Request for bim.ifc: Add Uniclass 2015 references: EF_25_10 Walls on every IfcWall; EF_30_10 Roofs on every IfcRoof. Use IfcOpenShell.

First a look at what the model holds.

```python
import ifcopenshell

model = ifcopenshell.open("bim.ifc")
print(model.schema)
print("classifications:", [c.Name for c in model.by_type("IfcClassification")])
for ifc_class in ("IfcDoor", "IfcRoof", "IfcStair", "IfcWall", "IfcWindow"):
    print(ifc_class, len(model.by_type(ifc_class)))
```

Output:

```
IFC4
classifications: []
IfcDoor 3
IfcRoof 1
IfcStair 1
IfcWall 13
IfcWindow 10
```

```python
import ifcopenshell
import ifcopenshell.api.classification

model = ifcopenshell.open("bim.ifc")

system = ifcopenshell.api.classification.add_classification(model, classification="Uniclass 2015")

codes = {
    "IfcWall": ("EF_25_10", "Walls"),
    "IfcRoof": ("EF_30_10", "Roofs"),
}
for ifc_class, (code, name) in codes.items():
    products = model.by_type(ifc_class)
    ifcopenshell.api.classification.add_reference(
        model, products=products, classification=system, identification=code, name=name
    )
    print(code, len(products))

model.write("bim_edited.ifc")
```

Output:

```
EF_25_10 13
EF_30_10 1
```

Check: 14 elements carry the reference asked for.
